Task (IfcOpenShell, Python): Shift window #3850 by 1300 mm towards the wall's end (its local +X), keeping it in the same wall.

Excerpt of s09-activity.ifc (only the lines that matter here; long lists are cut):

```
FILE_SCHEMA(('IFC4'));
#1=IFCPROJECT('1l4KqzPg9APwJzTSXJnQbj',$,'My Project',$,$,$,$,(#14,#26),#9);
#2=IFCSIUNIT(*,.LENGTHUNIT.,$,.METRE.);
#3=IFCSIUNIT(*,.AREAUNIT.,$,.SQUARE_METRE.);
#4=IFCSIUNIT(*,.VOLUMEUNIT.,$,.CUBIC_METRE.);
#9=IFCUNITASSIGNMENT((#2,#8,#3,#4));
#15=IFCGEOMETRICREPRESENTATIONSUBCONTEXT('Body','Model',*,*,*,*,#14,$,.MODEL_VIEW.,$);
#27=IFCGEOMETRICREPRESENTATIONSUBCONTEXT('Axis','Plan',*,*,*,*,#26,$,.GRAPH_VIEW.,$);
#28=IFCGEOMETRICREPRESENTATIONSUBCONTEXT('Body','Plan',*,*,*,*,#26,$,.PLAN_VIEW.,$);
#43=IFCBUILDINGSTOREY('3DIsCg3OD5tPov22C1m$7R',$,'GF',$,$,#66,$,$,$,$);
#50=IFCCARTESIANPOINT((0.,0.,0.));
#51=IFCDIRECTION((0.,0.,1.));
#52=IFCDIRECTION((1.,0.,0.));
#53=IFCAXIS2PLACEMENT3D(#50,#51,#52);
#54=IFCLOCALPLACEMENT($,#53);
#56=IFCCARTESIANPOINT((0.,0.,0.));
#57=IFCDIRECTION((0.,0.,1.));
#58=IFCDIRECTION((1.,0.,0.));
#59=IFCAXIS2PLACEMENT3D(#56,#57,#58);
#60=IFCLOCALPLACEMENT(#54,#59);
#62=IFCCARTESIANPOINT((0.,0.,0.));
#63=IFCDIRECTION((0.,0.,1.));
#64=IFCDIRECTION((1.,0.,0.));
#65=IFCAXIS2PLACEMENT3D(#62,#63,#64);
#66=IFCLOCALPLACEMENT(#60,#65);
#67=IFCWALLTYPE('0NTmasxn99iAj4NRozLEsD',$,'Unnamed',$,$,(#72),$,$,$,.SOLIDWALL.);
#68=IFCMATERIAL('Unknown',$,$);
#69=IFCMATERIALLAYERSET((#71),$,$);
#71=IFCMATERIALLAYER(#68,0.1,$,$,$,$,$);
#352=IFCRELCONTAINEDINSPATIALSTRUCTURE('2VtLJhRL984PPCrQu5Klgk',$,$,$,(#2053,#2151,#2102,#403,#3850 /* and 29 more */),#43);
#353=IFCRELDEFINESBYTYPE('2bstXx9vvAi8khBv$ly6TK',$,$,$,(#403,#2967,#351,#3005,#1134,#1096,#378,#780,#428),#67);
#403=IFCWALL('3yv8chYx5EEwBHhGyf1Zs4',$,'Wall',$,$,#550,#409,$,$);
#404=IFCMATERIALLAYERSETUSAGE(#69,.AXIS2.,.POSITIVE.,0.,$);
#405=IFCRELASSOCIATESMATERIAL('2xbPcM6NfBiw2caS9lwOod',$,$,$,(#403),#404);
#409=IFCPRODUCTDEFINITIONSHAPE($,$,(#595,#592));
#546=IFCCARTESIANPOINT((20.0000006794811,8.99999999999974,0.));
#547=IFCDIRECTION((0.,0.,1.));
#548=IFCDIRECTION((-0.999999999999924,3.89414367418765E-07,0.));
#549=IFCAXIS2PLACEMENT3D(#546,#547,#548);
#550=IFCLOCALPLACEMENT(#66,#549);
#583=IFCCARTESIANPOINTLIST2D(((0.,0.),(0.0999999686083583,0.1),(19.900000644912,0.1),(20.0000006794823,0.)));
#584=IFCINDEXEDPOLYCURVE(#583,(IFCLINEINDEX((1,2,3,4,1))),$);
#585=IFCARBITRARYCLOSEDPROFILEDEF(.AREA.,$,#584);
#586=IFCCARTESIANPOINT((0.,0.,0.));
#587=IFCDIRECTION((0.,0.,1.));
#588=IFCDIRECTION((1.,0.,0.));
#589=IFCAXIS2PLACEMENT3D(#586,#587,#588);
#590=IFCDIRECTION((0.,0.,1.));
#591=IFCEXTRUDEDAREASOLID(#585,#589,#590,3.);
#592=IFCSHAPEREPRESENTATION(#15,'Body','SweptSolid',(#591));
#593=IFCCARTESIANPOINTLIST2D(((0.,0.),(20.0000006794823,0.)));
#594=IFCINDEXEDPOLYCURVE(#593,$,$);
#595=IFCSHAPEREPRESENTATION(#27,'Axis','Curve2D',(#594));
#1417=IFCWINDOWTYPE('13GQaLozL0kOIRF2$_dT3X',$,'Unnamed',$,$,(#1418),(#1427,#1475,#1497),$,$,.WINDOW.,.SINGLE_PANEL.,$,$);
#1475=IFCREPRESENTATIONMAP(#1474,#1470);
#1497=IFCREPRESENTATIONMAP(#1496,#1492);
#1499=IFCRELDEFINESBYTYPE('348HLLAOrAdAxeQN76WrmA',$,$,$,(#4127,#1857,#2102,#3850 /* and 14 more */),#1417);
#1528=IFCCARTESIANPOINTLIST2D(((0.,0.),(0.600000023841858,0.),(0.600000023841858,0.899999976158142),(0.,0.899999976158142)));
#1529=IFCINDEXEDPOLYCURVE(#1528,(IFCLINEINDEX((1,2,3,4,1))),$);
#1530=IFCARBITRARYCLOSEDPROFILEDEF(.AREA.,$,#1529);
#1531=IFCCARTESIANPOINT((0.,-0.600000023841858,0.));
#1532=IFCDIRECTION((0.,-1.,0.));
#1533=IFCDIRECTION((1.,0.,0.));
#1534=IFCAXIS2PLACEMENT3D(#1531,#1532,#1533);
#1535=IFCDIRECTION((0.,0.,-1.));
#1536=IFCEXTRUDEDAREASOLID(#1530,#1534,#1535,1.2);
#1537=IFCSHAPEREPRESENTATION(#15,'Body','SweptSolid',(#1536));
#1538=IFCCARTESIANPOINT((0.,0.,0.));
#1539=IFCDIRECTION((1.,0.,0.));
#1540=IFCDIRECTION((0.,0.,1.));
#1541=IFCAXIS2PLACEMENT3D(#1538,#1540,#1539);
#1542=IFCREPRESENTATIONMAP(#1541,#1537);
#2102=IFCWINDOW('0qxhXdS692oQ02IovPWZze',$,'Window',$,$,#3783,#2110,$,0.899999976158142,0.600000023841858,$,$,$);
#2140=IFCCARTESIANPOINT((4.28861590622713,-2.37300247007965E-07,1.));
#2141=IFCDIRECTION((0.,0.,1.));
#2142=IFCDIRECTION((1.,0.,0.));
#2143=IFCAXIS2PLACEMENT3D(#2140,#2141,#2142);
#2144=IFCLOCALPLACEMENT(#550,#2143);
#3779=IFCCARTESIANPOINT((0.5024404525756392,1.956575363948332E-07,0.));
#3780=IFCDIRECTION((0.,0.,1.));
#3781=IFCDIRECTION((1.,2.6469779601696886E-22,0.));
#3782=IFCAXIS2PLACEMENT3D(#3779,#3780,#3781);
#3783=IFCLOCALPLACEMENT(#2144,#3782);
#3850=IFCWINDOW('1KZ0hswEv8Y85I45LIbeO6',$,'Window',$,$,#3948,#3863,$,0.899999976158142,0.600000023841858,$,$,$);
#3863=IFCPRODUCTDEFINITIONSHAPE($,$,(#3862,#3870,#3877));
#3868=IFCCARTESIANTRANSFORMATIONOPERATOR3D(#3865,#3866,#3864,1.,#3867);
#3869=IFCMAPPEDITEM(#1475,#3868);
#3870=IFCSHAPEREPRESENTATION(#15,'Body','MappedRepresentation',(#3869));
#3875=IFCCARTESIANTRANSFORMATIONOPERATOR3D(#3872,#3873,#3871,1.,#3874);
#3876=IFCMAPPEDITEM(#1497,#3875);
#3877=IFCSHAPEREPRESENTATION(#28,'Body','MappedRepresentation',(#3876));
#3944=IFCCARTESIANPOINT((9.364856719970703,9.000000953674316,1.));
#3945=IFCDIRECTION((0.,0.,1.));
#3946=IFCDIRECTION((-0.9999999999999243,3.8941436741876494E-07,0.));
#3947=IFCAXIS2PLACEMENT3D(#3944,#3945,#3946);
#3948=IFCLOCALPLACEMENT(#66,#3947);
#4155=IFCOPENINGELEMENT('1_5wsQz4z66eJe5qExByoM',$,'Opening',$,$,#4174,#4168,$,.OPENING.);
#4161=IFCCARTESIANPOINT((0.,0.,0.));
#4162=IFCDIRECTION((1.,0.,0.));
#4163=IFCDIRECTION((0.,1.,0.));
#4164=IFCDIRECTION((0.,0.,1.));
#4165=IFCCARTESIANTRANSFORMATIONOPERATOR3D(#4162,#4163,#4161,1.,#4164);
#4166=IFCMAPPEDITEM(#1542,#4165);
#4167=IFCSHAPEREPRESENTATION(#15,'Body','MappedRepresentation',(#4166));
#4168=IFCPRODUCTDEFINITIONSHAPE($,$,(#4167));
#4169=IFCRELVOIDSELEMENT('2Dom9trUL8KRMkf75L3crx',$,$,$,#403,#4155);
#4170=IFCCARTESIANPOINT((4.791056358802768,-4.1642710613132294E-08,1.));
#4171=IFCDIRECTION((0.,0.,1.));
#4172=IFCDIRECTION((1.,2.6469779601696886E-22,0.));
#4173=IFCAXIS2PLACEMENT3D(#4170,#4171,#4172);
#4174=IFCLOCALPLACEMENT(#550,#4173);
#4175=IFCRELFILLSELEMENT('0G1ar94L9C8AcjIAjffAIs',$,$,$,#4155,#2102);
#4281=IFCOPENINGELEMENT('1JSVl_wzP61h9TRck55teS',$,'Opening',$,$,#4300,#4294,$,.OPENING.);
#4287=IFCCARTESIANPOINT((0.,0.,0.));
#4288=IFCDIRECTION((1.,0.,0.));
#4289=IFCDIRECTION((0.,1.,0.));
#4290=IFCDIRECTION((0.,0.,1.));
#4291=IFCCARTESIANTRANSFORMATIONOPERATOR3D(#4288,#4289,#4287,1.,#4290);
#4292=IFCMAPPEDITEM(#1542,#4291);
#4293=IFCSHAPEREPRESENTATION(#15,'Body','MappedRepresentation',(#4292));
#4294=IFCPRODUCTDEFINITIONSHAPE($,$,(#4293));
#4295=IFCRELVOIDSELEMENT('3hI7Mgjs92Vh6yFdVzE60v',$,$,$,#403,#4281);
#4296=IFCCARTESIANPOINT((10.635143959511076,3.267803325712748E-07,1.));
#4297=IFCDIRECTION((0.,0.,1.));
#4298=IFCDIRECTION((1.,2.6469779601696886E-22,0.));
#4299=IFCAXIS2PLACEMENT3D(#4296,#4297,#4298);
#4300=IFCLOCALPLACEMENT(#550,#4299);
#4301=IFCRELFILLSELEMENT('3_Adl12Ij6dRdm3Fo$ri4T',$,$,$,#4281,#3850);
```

```python
import ifcopenshell
import ifcopenshell.api.geometry
import ifcopenshell.util.placement

model = ifcopenshell.open("s09-activity.ifc")

window = model.by_guid("1KZ0hswEv8Y85I45LIbeO6")
opening = window.FillsVoids[0].RelatingOpeningElement
wall = opening.VoidsElements[0].RelatingBuildingElement

wall_matrix = ifcopenshell.util.placement.get_local_placement(wall.ObjectPlacement)
shift = wall_matrix[:3, 0] * 1.3
before = ifcopenshell.util.placement.get_local_placement(window.ObjectPlacement)[:3, 3].copy()

# The window is not placed relative to its opening, so move both.
for product in (opening, window):
    matrix = ifcopenshell.util.placement.get_local_placement(product.ObjectPlacement)
    matrix[:3, 3] += shift
    ifcopenshell.api.geometry.edit_object_placement(model, product=product, matrix=matrix, is_si=False)

after = ifcopenshell.util.placement.get_local_placement(window.ObjectPlacement)[:3, 3]
print("window moved by", (after - before).round(3) + 0.0)

model.write("s09-activity_v2.ifc")
```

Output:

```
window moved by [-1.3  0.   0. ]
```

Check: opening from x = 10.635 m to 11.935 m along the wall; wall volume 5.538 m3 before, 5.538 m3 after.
